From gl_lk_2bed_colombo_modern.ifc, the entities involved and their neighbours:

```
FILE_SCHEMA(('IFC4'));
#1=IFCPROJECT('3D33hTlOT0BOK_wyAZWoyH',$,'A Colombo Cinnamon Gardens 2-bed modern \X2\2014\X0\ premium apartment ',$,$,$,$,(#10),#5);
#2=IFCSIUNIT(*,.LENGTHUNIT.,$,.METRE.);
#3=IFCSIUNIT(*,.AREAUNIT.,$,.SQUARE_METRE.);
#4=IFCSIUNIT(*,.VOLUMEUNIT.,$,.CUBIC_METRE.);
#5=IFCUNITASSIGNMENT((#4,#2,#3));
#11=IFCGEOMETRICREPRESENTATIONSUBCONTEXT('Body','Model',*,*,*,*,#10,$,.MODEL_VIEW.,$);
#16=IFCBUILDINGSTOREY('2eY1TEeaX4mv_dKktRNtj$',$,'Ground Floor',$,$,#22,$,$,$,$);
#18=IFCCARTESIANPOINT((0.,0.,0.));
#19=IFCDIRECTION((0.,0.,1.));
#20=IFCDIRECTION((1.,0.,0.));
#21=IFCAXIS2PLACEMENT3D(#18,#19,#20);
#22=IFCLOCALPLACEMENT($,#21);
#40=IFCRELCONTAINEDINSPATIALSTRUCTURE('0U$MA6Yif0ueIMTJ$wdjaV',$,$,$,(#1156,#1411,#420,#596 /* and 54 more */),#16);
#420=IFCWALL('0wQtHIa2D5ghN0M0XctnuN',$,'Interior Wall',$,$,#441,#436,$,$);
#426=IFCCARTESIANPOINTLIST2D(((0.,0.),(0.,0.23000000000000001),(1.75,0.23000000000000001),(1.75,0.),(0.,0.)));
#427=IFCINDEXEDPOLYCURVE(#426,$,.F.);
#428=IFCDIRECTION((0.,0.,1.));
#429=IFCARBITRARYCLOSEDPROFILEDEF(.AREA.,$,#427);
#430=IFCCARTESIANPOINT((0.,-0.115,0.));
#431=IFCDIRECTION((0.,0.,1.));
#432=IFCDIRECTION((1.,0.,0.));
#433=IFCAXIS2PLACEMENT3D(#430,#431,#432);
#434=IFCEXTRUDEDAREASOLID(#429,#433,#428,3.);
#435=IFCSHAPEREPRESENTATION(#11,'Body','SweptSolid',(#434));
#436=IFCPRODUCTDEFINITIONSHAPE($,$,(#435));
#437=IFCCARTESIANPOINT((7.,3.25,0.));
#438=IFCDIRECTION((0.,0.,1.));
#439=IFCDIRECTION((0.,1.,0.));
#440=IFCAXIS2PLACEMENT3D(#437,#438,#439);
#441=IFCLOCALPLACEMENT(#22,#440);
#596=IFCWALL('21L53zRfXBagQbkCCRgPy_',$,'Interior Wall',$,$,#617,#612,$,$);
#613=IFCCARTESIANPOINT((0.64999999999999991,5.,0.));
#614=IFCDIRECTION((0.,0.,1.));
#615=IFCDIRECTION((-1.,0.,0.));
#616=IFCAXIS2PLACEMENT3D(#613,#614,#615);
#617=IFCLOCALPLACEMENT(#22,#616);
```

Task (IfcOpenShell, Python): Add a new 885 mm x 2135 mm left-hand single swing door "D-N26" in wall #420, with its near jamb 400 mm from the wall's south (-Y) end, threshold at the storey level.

```python
import numpy as np
import ifcopenshell
import ifcopenshell.api.feature
import ifcopenshell.api.geometry
import ifcopenshell.api.root
import ifcopenshell.api.spatial
import ifcopenshell.geom
import ifcopenshell.util.element
import ifcopenshell.util.placement
import ifcopenshell.util.representation
import ifcopenshell.util.shape
import ifcopenshell.util.unit

model = ifcopenshell.open("gl_lk_2bed_colombo_modern.ifc")
unit_scale = ifcopenshell.util.unit.calculate_unit_scale(model)
settings = ifcopenshell.geom.settings()


def volume(element):
    """Net volume in cubic metres, openings subtracted."""
    shape = ifcopenshell.geom.create_shape(settings, element)
    return ifcopenshell.util.shape.get_volume(shape.geometry)


wall = model.by_guid("0wQtHIa2D5ghN0M0XctnuN")
storey = ifcopenshell.util.element.get_container(wall, ifc_class="IfcBuildingStorey")
context = ifcopenshell.util.representation.get_context(model, "Model", "Body", "MODEL_VIEW")
before = volume(wall)

width, height, from_end, sill = 0.885, 2.135, 0.4, 0.0  # metres

# The wall runs along its own X axis, and the end named is its -X end.
wall_shape = ifcopenshell.geom.create_shape(settings, wall)
x, y, z = ifcopenshell.util.shape.get_vertices(wall_shape.geometry).T
start = x.min() + from_end
face, thickness = float(y.min()), float(y.max() - y.min())
wall_matrix = ifcopenshell.util.placement.get_local_placement(wall.ObjectPlacement)
level = ifcopenshell.util.placement.get_local_placement(storey.ObjectPlacement)[2, 3]


def in_wall(x, y):
    """Placement at x, y metres in the wall's axes, at sill height."""
    matrix = wall_matrix.copy()
    matrix[:, 3] = wall_matrix @ np.array([x / unit_scale, y / unit_scale, 0.0, 1.0])
    matrix[2, 3] = level + sill / unit_scale
    return matrix


# Opening: a box that overshoots both wall faces by 50 mm.
opening = ifcopenshell.api.root.create_entity(model, ifc_class="IfcOpeningElement", predefined_type="OPENING")
box = ifcopenshell.api.geometry.add_wall_representation(
    model, context=context, length=width, height=height, thickness=thickness + 0.1
)
ifcopenshell.api.geometry.assign_representation(model, product=opening, representation=box)
ifcopenshell.api.geometry.edit_object_placement(model, product=opening, matrix=in_wall(start, face - 0.05), is_si=False)
ifcopenshell.api.feature.add_feature(model, feature=opening, element=wall)

door = ifcopenshell.api.root.create_entity(model, ifc_class="IfcDoor", name="D-N26", predefined_type="DOOR")
door.OverallWidth, door.OverallHeight = width / unit_scale, height / unit_scale
door.OperationType = "SINGLE_SWING_LEFT"
body = ifcopenshell.api.geometry.add_door_representation(
    model,
    context=context,
    overall_width=door.OverallWidth,
    overall_height=door.OverallHeight,
    operation_type="SINGLE_SWING_LEFT",
    lining_properties={"LiningDepth": thickness / unit_scale, "ThresholdDepth": thickness / unit_scale},
)
ifcopenshell.api.geometry.assign_representation(model, product=door, representation=body)
ifcopenshell.api.spatial.assign_container(model, products=[door], relating_structure=storey)
ifcopenshell.api.feature.add_filling(model, opening=opening, element=door)

# The lining spans the wall, so the door starts at the wall face.
ifcopenshell.api.geometry.edit_object_placement(model, product=door, matrix=in_wall(start, face), is_si=False)

after = volume(wall)

print(f"wall volume {before:.3f} -> {after:.3f} m3")

model.write("gl_lk_2bed_colombo_modern_rev.ifc")
```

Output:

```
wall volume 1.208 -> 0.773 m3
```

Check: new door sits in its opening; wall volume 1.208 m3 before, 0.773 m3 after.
